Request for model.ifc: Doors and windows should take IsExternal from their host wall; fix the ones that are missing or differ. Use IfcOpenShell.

First a look at what the model holds.

```python
import ifcopenshell
import ifcopenshell.util.element

model = ifcopenshell.open("model.ifc")
print(model.schema)
seen = {}
for e in model.by_type("IfcDoor") + model.by_type("IfcWindow"):
    if not e.FillsVoids:
        continue
    host = e.FillsVoids[0].RelatingOpeningElement.VoidsElements[0].RelatingBuildingElement
    own = ifcopenshell.util.element.get_pset(e, f"Pset_{e.is_a()[3:].removesuffix('StandardCase')}Common", "IsExternal")
    wall = ifcopenshell.util.element.get_pset(host, "Pset_WallCommon", "IsExternal")
    seen[e.is_a(), own, wall] = seen.get((e.is_a(), own, wall), 0) + 1
for (cls, own, wall), count in sorted(seen.items(), key=str):
    print(count, cls, "IsExternal:", own, "| host wall:", wall)
```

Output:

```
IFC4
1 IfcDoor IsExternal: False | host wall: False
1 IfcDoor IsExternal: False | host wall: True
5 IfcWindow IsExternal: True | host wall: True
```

```python
import ifcopenshell
import ifcopenshell.api.pset
import ifcopenshell.util.element

model = ifcopenshell.open("model.ifc")

count = 0
for ifc_class, pset_name in (("IfcDoor", "Pset_DoorCommon"), ("IfcWindow", "Pset_WindowCommon")):
    for e in model.by_type(ifc_class):
        if not e.FillsVoids:
            continue
        host = e.FillsVoids[0].RelatingOpeningElement.VoidsElements[0].RelatingBuildingElement
        external = ifcopenshell.util.element.get_pset(host, "Pset_WallCommon", "IsExternal")
        if external is None or ifcopenshell.util.element.get_pset(e, pset_name, "IsExternal") == external:
            continue
        pset = ifcopenshell.api.pset.add_pset(model, product=e, name=pset_name)
        ifcopenshell.api.pset.edit_pset(model, pset=pset, properties={"IsExternal": external})
        count += 1

print(count, "updated")

model.write("model_updated.ifc")
```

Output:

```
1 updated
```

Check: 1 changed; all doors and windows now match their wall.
